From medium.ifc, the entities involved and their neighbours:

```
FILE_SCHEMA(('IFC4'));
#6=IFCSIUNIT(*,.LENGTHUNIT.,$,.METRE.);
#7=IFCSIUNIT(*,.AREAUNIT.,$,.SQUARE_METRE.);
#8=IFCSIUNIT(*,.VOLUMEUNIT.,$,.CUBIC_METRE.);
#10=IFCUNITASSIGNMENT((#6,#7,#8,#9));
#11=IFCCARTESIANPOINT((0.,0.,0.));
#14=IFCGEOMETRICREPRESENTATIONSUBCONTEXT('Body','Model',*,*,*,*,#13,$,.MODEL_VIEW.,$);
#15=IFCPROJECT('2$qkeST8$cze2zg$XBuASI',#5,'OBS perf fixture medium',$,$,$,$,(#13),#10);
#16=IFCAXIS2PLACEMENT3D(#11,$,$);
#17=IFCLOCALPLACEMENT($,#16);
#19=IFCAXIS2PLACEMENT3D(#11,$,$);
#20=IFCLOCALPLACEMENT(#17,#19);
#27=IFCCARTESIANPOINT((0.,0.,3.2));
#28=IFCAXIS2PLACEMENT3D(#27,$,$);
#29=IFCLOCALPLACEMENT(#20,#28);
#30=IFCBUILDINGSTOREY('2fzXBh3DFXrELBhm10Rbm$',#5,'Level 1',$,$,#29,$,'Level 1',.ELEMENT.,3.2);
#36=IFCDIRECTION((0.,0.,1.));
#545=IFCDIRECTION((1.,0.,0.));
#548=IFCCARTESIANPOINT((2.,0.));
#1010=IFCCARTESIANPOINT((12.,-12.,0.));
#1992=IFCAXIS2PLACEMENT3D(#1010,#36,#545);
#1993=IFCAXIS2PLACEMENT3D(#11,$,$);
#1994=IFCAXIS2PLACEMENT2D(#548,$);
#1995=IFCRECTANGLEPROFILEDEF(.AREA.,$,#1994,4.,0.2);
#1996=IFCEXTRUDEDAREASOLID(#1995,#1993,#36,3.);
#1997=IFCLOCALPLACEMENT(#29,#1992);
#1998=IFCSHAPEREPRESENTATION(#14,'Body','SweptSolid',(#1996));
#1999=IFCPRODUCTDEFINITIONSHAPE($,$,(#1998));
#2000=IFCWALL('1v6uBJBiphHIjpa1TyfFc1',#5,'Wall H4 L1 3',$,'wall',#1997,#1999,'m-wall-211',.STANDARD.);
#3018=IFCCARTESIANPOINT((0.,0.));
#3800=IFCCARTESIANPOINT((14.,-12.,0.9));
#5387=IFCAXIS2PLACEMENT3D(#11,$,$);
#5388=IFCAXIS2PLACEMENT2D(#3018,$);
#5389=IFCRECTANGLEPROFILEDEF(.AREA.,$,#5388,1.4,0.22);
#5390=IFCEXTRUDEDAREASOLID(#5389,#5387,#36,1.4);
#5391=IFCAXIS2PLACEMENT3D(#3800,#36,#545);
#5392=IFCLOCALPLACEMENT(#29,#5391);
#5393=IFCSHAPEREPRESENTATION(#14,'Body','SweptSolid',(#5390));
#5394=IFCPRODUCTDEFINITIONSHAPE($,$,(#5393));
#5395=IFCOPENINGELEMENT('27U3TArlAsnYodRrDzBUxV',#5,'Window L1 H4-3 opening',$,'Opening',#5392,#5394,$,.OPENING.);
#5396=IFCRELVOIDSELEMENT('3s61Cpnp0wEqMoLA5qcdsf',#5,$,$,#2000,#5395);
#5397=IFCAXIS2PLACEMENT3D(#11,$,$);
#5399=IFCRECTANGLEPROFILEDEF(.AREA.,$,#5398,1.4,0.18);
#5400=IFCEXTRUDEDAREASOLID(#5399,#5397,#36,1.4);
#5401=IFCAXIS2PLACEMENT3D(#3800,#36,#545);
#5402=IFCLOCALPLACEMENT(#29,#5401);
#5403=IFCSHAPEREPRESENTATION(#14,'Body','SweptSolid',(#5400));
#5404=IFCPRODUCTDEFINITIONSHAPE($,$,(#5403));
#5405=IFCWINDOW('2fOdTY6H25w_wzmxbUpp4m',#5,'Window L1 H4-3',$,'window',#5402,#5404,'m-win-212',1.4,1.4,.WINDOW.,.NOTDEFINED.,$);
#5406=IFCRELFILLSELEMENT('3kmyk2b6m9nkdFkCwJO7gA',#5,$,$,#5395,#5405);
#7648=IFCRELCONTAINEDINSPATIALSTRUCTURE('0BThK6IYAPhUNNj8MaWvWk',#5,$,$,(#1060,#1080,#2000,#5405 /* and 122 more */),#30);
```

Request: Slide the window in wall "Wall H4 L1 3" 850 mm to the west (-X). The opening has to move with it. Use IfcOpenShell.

```python
import ifcopenshell
import ifcopenshell.api.geometry
import ifcopenshell.util.placement

model = ifcopenshell.open("medium.ifc")

window = model.by_guid("2fOdTY6H25w_wzmxbUpp4m")
opening = window.FillsVoids[0].RelatingOpeningElement
wall = opening.VoidsElements[0].RelatingBuildingElement

wall_matrix = ifcopenshell.util.placement.get_local_placement(wall.ObjectPlacement)
shift = wall_matrix[:3, 0] * -0.85
before = ifcopenshell.util.placement.get_local_placement(window.ObjectPlacement)[:3, 3].copy()

# The window is not placed relative to its opening, so move both.
for product in (opening, window):
    matrix = ifcopenshell.util.placement.get_local_placement(product.ObjectPlacement)
    matrix[:3, 3] += shift
    ifcopenshell.api.geometry.edit_object_placement(model, product=product, matrix=matrix, is_si=False)

after = ifcopenshell.util.placement.get_local_placement(window.ObjectPlacement)[:3, 3]
print("window moved by", (after - before).round(3) + 0.0)

model.write("medium_v2.ifc")
```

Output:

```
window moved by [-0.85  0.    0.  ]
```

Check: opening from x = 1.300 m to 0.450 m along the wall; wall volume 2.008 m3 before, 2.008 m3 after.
